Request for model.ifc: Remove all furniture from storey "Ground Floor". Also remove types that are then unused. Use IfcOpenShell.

First a look at what the model holds.

```python
import ifcopenshell
import ifcopenshell.util.element

model = ifcopenshell.open("model.ifc")
print(model.schema)
storey = next(s for s in model.by_type("IfcBuildingStorey") if s.Name == "Ground Floor")
furniture = [e for e in ifcopenshell.util.element.get_decomposition(storey) if e.is_a("IfcFurnishingElement")]
seen = {}
for e in furniture:
    element_type = ifcopenshell.util.element.get_type(e)
    name = element_type.Name if element_type not in (None, e) else None
    seen[name] = seen.get(name, 0) + 1
for name, count in sorted(seen.items(), key=str):
    print(count, "x", name)
```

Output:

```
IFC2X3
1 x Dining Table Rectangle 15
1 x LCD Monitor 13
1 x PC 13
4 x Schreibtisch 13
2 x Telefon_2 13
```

```python
import ifcopenshell
import ifcopenshell.api.root
import ifcopenshell.util.element

model = ifcopenshell.open("model.ifc")

storey = next(s for s in model.by_type("IfcBuildingStorey") if s.Name == "Ground Floor")
furniture = [e for e in ifcopenshell.util.element.get_decomposition(storey) if e.is_a("IfcFurnishingElement")]
types = {ifcopenshell.util.element.get_type(e) for e in furniture} - {None, *furniture}

for e in furniture:
    ifcopenshell.api.root.remove_product(model, product=e)
print(len(furniture), "removed")

unused = [t for t in types if not ifcopenshell.util.element.get_types(t)]
for t in unused:
    ifcopenshell.api.root.remove_product(model, product=t)
print(len(unused), "unused types removed")

model.write("model_edited.ifc")
```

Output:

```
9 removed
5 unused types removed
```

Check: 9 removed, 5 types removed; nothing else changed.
